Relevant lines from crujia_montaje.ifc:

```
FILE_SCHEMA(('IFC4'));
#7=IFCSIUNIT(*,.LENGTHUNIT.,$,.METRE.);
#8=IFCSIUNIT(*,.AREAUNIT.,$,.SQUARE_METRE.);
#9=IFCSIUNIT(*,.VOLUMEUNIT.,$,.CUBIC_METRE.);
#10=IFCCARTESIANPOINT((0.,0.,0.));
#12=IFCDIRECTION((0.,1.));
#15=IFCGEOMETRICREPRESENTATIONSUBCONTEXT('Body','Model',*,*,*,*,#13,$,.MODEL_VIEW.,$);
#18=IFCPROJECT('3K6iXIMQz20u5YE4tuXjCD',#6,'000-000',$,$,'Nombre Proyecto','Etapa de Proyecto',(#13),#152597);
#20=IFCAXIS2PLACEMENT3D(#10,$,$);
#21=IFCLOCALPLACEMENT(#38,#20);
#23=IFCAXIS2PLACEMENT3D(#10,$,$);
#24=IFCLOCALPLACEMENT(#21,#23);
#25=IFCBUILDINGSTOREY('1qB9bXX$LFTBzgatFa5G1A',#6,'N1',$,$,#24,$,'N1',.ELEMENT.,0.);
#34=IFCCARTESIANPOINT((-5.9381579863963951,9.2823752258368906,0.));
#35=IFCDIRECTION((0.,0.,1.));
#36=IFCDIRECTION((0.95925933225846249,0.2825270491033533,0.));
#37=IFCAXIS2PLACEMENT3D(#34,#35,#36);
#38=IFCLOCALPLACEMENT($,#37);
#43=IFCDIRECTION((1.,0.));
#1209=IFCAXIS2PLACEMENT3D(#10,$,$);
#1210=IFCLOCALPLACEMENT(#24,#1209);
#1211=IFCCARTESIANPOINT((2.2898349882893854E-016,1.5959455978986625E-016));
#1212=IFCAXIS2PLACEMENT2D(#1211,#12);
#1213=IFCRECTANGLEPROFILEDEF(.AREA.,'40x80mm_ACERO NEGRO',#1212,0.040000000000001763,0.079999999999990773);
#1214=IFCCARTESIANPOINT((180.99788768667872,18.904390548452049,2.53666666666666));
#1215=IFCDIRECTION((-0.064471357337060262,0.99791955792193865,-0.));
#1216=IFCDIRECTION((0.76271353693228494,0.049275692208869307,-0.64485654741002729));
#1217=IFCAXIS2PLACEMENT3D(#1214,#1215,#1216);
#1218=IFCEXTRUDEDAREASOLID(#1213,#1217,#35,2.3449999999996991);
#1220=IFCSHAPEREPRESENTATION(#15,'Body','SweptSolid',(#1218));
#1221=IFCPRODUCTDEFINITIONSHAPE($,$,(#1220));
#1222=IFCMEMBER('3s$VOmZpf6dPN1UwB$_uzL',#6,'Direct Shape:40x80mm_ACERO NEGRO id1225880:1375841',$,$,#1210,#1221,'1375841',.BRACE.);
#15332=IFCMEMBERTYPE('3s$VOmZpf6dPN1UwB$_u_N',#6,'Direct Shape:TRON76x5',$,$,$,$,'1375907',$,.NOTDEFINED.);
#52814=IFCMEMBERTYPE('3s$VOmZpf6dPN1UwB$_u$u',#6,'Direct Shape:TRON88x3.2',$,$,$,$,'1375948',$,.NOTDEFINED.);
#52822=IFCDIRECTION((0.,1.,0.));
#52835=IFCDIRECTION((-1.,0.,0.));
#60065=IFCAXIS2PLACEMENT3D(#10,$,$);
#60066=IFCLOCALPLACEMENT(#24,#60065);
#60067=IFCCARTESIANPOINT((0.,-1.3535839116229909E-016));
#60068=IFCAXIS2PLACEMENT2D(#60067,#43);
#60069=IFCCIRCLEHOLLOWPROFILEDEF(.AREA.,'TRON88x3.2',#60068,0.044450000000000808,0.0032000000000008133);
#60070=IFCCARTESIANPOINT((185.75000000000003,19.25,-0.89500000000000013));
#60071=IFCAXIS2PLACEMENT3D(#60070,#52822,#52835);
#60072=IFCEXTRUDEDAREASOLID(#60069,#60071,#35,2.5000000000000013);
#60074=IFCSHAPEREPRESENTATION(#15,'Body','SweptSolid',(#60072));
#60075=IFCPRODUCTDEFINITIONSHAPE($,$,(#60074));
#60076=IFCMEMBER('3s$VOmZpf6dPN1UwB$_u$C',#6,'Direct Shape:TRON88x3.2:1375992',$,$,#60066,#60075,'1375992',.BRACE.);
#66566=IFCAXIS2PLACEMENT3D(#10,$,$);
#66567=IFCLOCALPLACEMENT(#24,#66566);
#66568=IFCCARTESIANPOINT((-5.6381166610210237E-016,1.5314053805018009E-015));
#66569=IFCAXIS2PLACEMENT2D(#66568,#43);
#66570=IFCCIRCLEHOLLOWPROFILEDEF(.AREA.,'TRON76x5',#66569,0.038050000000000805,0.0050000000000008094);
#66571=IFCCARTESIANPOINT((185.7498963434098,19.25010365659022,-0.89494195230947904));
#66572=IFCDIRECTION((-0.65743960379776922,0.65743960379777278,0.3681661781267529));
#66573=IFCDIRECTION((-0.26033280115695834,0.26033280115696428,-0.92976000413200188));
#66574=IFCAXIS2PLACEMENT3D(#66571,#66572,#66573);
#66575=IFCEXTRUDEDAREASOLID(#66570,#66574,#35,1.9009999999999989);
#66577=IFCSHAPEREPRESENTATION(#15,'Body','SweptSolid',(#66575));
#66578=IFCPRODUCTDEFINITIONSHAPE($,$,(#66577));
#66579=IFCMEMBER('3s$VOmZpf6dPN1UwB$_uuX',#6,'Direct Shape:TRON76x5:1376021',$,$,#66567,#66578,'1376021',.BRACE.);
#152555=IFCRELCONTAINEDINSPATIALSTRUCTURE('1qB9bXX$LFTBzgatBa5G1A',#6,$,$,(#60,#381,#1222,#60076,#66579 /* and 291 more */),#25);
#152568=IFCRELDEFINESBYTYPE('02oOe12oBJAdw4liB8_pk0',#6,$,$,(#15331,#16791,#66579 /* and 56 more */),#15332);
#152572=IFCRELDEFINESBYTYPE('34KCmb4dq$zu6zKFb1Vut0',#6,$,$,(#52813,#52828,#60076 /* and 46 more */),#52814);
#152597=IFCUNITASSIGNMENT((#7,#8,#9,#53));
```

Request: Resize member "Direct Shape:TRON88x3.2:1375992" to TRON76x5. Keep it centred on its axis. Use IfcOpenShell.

```python
import ifcopenshell
import ifcopenshell.api.type
import ifcopenshell.util.element
import ifcopenshell.util.representation

model = ifcopenshell.open("crujia_montaje.ifc")

member = model.by_guid("3s$VOmZpf6dPN1UwB$_u$C")
source = next(p for p in model.by_type("IfcCircleHollowProfileDef") if p.ProfileName == "TRON76x5")

body = ifcopenshell.util.representation.get_representation(member, "Model", "Body")
solid = body.Items[0]
old_profile = solid.SweptArea

# Copy the section's sizes but keep this member's own profile position.
profile = ifcopenshell.util.element.copy(model, source)
profile.Position = old_profile.Position
solid.SweptArea = profile
if not model.get_total_inverses(old_profile):
    ifcopenshell.util.element.remove_deep2(model, old_profile)

new_type = model.by_id(15332)
ifcopenshell.api.type.assign_type(
    model, related_objects=[member], relating_type=new_type, should_map_representations=False
)
member.Name = member.Name.replace("TRON88x3.2", "TRON76x5")

print(solid.SweptArea)

model.write("crujia_montaje_edited.ifc")
```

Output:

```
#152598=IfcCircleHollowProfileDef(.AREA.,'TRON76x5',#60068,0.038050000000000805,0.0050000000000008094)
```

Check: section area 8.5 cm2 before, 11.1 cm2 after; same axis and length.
